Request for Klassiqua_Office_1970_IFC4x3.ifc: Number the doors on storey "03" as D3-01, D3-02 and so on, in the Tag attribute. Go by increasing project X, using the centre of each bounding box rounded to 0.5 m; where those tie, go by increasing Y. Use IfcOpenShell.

First a look at what the model holds.

```python
import ifcopenshell
import ifcopenshell.util.element
import ifcopenshell.util.placement

model = ifcopenshell.open("Klassiqua_Office_1970_IFC4x3.ifc")
print(model.schema)
storey = next(s for s in model.by_type("IfcBuildingStorey") if s.Name == "03")
doors = [e for e in ifcopenshell.util.element.get_decomposition(storey) if e.is_a("IfcDoor")]
for e in sorted(doors, key=lambda e: e.id()):
    origin = ifcopenshell.util.placement.get_local_placement(e.ObjectPlacement)[:3, 3]
    print(e.id(), e.Tag, e.Name, origin.round(2) + 0.0, sep=" | ")
```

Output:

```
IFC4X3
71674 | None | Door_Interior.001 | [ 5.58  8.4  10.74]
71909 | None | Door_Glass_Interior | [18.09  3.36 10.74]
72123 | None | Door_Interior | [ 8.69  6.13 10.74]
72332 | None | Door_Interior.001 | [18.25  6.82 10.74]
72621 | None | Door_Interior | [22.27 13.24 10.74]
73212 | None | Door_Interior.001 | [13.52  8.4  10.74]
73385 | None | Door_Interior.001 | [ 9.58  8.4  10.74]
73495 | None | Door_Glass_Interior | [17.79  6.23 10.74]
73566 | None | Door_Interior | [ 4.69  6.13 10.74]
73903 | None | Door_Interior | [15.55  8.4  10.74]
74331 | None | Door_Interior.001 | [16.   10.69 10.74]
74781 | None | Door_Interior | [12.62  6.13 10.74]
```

```python
import ifcopenshell
import ifcopenshell.geom
import ifcopenshell.util.element
import ifcopenshell.util.shape

model = ifcopenshell.open("Klassiqua_Office_1970_IFC4x3.ifc")
settings = ifcopenshell.geom.settings()
settings.set("use-world-coords", True)


def centre(element):
    shape = ifcopenshell.geom.create_shape(settings, element)
    return ifcopenshell.util.shape.get_bbox_centroid(shape.geometry)


storey = next(s for s in model.by_type("IfcBuildingStorey") if s.Name == "03")
doors = [e for e in ifcopenshell.util.element.get_decomposition(storey) if e.is_a("IfcDoor")]

# Insertion points can sit at a corner or the storey origin, so sort by the geometry (in metres).
centres = {e: centre(e) for e in doors}
doors.sort(key=lambda e: (round(centres[e][0] / 0.5), centres[e][1]))

for i, e in enumerate(doors, start=1):
    number = f"D3-{i:02d}"
    e.Tag = number
    print(e.id(), number)

model.write("Klassiqua_Office_1970_IFC4x3_updated.ifc")
```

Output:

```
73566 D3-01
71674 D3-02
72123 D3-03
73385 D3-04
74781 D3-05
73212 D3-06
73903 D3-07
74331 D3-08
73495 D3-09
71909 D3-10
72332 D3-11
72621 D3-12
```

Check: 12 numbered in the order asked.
